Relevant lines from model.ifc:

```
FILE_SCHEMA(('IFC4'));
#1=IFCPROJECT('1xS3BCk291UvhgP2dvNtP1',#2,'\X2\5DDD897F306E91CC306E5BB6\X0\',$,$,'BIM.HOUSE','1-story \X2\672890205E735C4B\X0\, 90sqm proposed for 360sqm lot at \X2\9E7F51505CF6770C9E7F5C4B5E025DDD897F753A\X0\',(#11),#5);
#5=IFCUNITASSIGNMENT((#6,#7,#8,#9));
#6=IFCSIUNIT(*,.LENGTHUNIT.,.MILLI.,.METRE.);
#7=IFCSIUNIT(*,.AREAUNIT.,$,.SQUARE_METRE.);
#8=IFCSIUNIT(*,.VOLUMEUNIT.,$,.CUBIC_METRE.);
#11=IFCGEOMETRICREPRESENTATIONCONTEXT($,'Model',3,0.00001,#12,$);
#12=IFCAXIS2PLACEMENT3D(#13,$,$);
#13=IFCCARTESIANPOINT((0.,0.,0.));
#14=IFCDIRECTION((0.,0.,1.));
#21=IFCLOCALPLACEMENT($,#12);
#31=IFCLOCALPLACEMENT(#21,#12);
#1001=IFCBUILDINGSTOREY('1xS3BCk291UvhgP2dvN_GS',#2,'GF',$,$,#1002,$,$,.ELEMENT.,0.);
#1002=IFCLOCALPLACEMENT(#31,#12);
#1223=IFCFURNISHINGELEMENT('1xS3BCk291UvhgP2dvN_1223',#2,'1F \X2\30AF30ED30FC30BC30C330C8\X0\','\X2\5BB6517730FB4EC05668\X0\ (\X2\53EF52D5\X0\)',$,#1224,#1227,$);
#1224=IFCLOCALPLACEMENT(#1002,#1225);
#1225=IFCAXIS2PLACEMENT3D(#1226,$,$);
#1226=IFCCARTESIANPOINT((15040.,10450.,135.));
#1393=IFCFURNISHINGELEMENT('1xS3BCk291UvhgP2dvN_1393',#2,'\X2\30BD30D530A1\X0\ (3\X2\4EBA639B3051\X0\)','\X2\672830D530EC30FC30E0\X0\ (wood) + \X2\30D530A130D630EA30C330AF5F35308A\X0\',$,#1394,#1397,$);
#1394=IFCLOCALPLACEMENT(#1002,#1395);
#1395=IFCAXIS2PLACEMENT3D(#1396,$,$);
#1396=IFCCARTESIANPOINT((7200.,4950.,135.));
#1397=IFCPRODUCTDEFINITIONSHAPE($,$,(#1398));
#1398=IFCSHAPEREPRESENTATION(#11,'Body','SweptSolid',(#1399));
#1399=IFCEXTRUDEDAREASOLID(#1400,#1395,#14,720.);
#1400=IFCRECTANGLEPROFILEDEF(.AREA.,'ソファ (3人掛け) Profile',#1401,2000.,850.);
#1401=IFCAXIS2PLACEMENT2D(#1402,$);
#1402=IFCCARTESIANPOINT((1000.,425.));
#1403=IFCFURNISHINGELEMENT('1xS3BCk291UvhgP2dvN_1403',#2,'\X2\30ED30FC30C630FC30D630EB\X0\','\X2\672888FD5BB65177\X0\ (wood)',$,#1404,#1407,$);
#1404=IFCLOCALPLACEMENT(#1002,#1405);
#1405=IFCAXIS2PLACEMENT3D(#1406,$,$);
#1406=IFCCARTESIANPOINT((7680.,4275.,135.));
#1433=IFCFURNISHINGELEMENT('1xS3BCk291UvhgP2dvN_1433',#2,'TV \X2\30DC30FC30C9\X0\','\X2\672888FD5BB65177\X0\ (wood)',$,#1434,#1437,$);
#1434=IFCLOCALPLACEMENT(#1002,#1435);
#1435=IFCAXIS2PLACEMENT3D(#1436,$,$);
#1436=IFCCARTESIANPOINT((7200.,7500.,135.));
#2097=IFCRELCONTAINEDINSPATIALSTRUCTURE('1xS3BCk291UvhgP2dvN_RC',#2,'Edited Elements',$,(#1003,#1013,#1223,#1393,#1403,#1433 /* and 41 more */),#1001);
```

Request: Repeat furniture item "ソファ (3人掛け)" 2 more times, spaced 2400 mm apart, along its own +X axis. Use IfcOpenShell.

```python
import ifcopenshell
import ifcopenshell.api.geometry
import ifcopenshell.api.root
import ifcopenshell.util.element
import ifcopenshell.util.placement
import ifcopenshell.util.unit

model = ifcopenshell.open("model.ifc")
unit_scale = ifcopenshell.util.unit.calculate_unit_scale(model)


def reuse_history(source, copy):
    """copy_class also copies each property set's owner history, people and application; keep the originals."""
    for rel in copy.IsDefinedBy:
        if rel.is_a("IfcRelDefinesByProperties") and (history := rel.RelatingPropertyDefinition.OwnerHistory):
            rel.RelatingPropertyDefinition.OwnerHistory = source.OwnerHistory
            ifcopenshell.util.element.remove_deep2(model, history)


source = model.by_guid("1xS3BCk291UvhgP2dvN_1393")
base = ifcopenshell.util.placement.get_local_placement(source.ObjectPlacement)
step = base[:3, 0] * 2.4 / unit_scale

for i in range(1, 3):
    copy = ifcopenshell.api.root.copy_class(model, product=source)
    copy.Representation = ifcopenshell.util.element.copy_deep(
        model, source.Representation, exclude=["IfcGeometricRepresentationContext", "IfcRepresentationMap"]
    )
    reuse_history(source, copy)
    matrix = base.copy()
    matrix[:3, 3] += i * step
    print("added at", matrix[:3, 3].round(3) + 0.0)
    ifcopenshell.api.geometry.edit_object_placement(model, product=copy, matrix=matrix, is_si=False)

model.write("model_edited.ifc")
```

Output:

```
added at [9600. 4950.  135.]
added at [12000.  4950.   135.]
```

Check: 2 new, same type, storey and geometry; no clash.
